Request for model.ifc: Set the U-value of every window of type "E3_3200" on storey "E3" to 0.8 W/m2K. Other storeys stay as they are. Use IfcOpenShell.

First a look at what the model holds.

```python
import ifcopenshell
import ifcopenshell.util.element

model = ifcopenshell.open("model.ifc")
print(model.schema)
storey = next(s for s in model.by_type("IfcBuildingStorey") if s.Name == "E3")
windows = [e for e in ifcopenshell.util.element.get_decomposition(storey) if e.is_a("IfcWindow")]
seen = {}
for e in windows:
    element_type = ifcopenshell.util.element.get_type(e)
    key = (element_type.Name if element_type != e and element_type else None, ifcopenshell.util.element.get_pset(e, "Pset_WindowCommon", "ThermalTransmittance"))
    seen[key] = seen.get(key, 0) + 1
for (name, value), count in sorted(seen.items(), key=str):
    print(count, "x", name, "|", value)
```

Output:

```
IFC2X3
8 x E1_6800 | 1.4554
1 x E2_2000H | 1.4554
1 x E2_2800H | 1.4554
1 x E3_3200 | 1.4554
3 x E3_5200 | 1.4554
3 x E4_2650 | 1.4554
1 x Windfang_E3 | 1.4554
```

```python
import ifcopenshell
import ifcopenshell.api.pset
import ifcopenshell.util.element

model = ifcopenshell.open("model.ifc")

storey = next(s for s in model.by_type("IfcBuildingStorey") if s.Name == "E3")
windows = [e for e in ifcopenshell.util.element.get_decomposition(storey) if e.is_a("IfcWindow")]

count = 0
for e in windows:
    element_type = ifcopenshell.util.element.get_type(e)
    if element_type in (None, e) or element_type.Name != "E3_3200":
        continue
    # add_pset returns the element's existing set when there is one.
    pset = ifcopenshell.api.pset.add_pset(model, product=e, name="Pset_WindowCommon")
    ifcopenshell.api.pset.edit_pset(model, pset=pset, properties={"ThermalTransmittance": 0.8})
    count += 1

print(count, "windows updated")

model.write("model_rev.ifc")
```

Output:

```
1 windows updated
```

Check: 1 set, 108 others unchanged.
